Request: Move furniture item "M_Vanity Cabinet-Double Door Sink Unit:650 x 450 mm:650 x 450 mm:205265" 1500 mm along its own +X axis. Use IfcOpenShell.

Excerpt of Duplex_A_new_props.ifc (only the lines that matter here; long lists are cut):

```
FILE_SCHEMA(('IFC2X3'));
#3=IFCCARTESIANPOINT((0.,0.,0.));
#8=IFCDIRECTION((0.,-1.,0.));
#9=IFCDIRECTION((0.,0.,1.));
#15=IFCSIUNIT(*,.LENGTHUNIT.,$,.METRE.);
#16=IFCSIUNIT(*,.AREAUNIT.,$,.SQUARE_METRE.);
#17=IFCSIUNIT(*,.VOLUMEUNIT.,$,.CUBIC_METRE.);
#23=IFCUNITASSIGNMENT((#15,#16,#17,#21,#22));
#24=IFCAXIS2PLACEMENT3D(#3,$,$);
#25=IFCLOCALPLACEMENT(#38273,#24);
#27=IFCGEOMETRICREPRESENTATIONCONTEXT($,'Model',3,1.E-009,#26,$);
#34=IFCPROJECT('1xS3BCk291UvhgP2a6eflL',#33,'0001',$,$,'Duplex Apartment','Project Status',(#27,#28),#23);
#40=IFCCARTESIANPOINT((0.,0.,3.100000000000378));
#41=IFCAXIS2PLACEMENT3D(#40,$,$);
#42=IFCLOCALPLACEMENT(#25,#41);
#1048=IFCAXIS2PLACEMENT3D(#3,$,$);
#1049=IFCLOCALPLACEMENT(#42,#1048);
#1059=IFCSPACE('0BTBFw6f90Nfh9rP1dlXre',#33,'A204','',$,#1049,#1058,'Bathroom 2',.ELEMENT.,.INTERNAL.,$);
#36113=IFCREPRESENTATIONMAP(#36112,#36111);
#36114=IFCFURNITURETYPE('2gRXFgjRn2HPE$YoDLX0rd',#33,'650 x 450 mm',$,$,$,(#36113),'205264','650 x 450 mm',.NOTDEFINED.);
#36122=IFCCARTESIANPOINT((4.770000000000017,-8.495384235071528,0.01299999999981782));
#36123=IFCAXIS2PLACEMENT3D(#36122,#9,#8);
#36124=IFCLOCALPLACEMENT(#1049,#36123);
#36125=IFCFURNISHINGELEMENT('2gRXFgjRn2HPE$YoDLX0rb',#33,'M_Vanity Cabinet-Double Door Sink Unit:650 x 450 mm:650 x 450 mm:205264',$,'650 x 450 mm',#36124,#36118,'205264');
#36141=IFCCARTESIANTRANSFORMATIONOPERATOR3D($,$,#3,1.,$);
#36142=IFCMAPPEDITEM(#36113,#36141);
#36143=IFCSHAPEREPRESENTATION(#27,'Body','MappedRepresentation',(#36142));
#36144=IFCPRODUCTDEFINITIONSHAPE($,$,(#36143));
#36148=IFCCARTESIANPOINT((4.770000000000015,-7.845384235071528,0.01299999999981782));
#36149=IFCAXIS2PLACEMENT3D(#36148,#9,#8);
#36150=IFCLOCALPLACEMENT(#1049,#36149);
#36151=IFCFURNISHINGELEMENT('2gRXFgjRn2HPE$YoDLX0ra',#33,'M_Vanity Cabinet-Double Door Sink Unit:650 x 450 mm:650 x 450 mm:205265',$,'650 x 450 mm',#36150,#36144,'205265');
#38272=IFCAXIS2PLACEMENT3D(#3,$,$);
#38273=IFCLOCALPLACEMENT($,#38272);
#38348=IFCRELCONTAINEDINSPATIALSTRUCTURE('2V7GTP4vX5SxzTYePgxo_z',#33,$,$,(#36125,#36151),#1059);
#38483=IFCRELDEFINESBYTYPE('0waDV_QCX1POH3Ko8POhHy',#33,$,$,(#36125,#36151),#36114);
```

```python
import ifcopenshell
import ifcopenshell.api.geometry
import ifcopenshell.util.placement

model = ifcopenshell.open("Duplex_A_new_props.ifc")

item = model.by_id(36151)
matrix = ifcopenshell.util.placement.get_local_placement(item.ObjectPlacement)
matrix[:3, 3] += matrix[:3, 0] * 1.5
ifcopenshell.api.geometry.edit_object_placement(model, product=item, matrix=matrix, is_si=False)

print(ifcopenshell.util.placement.get_local_placement(item.ObjectPlacement).round(3) + 0.0)

model.write("Duplex_A_new_props_rev.ifc")
```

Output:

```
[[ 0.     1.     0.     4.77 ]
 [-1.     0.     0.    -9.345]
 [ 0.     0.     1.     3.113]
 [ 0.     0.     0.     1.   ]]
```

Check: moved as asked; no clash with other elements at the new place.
